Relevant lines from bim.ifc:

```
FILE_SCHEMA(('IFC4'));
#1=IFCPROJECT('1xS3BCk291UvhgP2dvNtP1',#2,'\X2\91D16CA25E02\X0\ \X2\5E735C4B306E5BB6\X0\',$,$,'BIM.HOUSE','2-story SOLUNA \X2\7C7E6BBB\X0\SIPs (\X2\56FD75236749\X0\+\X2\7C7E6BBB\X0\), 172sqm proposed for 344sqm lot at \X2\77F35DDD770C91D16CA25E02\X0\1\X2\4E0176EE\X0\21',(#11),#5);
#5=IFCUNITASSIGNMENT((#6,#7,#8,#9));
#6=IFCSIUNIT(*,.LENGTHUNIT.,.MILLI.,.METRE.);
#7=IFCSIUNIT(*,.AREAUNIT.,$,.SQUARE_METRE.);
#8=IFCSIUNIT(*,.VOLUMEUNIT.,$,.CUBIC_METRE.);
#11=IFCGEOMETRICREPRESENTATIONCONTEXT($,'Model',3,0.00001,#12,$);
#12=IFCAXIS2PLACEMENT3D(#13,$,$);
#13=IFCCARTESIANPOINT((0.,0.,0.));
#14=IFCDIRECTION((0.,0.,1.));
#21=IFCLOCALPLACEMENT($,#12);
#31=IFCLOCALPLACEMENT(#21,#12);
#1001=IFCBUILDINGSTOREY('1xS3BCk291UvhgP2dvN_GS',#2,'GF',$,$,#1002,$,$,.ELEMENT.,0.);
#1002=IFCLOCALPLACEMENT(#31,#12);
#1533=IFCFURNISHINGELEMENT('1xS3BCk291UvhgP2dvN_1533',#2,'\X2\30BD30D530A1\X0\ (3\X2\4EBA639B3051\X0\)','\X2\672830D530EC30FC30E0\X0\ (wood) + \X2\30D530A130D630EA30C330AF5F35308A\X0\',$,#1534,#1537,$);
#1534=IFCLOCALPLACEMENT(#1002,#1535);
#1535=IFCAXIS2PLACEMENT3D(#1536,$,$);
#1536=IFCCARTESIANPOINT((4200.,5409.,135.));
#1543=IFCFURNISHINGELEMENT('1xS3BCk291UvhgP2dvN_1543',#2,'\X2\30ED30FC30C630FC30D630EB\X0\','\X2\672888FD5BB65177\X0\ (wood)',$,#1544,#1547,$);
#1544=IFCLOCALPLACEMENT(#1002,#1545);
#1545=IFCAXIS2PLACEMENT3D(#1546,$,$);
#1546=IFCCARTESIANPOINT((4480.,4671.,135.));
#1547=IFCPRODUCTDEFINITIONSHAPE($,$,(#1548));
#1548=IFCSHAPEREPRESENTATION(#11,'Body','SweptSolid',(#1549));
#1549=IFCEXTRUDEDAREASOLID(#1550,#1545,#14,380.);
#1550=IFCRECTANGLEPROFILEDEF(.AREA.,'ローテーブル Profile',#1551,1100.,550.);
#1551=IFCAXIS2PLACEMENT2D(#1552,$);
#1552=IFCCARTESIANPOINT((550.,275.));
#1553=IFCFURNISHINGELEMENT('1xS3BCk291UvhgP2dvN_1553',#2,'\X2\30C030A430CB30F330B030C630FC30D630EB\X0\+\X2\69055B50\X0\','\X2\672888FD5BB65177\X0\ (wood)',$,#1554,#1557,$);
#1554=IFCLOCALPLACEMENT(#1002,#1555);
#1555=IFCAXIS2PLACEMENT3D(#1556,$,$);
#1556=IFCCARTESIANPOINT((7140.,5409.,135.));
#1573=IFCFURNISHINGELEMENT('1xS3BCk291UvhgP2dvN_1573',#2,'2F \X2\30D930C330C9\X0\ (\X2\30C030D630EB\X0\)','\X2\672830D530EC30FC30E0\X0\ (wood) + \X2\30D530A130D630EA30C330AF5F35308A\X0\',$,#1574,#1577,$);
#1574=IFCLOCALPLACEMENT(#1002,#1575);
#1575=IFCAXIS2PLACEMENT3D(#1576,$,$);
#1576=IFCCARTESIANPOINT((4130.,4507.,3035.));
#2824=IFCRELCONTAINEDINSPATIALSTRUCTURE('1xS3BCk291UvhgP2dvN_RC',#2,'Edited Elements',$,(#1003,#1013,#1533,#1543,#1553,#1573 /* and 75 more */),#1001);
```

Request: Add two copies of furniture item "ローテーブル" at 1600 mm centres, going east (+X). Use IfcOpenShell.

```python
import numpy as np
import ifcopenshell
import ifcopenshell.api.geometry
import ifcopenshell.api.root
import ifcopenshell.util.element
import ifcopenshell.util.placement

model = ifcopenshell.open("bim.ifc")


def reuse_history(source, copy):
    """copy_class also copies each property set's owner history, people and application; keep the originals."""
    for rel in copy.IsDefinedBy:
        if rel.is_a("IfcRelDefinesByProperties") and (history := rel.RelatingPropertyDefinition.OwnerHistory):
            rel.RelatingPropertyDefinition.OwnerHistory = source.OwnerHistory
            ifcopenshell.util.element.remove_deep2(model, history)


source = model.by_guid("1xS3BCk291UvhgP2dvN_1543")
base = ifcopenshell.util.placement.get_local_placement(source.ObjectPlacement)
step = np.array([1.0, 0.0, 0.0]) * 1600.0

for i in range(1, 3):
    copy = ifcopenshell.api.root.copy_class(model, product=source)
    copy.Representation = ifcopenshell.util.element.copy_deep(
        model, source.Representation, exclude=["IfcGeometricRepresentationContext", "IfcRepresentationMap"]
    )
    reuse_history(source, copy)
    matrix = base.copy()
    matrix[:3, 3] += i * step
    print("added at", matrix[:3, 3].round(3) + 0.0)
    ifcopenshell.api.geometry.edit_object_placement(model, product=copy, matrix=matrix, is_si=False)

model.write("bim-out.ifc")
```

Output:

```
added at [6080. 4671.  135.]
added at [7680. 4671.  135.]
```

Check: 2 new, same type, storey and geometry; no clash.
